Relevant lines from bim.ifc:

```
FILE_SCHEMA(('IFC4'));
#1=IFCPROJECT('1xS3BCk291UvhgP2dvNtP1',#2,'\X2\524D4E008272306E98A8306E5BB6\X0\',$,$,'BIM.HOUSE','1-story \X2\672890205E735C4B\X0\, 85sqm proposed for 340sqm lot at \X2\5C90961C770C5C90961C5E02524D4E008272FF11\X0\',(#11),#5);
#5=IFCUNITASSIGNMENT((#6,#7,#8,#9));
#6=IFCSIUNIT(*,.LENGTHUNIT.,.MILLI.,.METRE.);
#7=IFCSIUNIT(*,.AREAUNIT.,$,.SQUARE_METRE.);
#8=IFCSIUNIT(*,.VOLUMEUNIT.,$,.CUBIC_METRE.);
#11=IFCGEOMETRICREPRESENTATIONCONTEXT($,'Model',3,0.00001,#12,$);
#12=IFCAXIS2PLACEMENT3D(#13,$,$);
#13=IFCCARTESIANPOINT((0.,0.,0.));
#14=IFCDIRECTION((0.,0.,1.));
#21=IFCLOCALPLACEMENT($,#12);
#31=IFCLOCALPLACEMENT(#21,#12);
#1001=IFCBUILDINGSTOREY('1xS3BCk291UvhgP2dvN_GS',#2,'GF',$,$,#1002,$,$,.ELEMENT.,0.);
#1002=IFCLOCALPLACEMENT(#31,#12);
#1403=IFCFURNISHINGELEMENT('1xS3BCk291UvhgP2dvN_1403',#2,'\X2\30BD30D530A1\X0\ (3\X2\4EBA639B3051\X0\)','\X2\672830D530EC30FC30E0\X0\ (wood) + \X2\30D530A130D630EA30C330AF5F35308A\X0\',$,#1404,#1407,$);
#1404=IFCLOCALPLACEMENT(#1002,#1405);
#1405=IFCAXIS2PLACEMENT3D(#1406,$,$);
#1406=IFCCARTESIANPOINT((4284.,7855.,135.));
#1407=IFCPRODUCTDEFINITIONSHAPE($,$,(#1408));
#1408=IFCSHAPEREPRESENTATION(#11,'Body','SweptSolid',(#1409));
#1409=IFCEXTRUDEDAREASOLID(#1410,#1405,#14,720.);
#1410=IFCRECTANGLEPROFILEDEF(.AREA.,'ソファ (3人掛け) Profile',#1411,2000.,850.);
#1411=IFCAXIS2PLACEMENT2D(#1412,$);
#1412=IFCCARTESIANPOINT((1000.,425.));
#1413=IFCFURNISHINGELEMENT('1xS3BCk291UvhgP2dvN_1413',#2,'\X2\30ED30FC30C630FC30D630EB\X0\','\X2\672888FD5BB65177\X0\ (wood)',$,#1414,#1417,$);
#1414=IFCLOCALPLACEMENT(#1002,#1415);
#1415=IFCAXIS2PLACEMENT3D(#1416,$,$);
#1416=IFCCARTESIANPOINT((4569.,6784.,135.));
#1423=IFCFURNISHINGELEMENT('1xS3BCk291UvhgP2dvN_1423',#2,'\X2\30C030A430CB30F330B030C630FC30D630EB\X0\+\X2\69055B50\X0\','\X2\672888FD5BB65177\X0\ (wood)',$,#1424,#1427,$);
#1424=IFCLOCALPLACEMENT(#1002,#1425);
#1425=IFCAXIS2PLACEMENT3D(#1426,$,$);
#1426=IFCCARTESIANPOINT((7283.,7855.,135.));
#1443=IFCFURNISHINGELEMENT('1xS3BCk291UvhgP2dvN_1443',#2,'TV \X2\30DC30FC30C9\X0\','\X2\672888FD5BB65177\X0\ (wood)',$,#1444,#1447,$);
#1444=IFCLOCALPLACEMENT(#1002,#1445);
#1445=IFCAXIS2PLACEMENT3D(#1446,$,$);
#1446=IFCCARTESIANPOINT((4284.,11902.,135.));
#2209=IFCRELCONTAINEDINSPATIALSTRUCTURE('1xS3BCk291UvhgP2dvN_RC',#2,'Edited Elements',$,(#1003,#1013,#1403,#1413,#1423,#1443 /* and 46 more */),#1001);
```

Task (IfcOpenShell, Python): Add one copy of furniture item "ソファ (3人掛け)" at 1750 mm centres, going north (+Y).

```python
import numpy as np
import ifcopenshell
import ifcopenshell.api.geometry
import ifcopenshell.api.root
import ifcopenshell.util.element
import ifcopenshell.util.placement
import ifcopenshell.util.unit

model = ifcopenshell.open("bim.ifc")
unit_scale = ifcopenshell.util.unit.calculate_unit_scale(model)


def reuse_history(source, copy):
    """copy_class also copies each property set's owner history, people and application; keep the originals."""
    for rel in copy.IsDefinedBy:
        if rel.is_a("IfcRelDefinesByProperties") and (history := rel.RelatingPropertyDefinition.OwnerHistory):
            rel.RelatingPropertyDefinition.OwnerHistory = source.OwnerHistory
            ifcopenshell.util.element.remove_deep2(model, history)


source = model.by_id(1403)
base = ifcopenshell.util.placement.get_local_placement(source.ObjectPlacement)
step = np.array([0.0, 1.0, 0.0]) * 1.75 / unit_scale

for i in range(1, 2):
    copy = ifcopenshell.api.root.copy_class(model, product=source)
    copy.Representation = ifcopenshell.util.element.copy_deep(
        model, source.Representation, exclude=["IfcGeometricRepresentationContext", "IfcRepresentationMap"]
    )
    reuse_history(source, copy)
    matrix = base.copy()
    matrix[:3, 3] += i * step
    print("added at", matrix[:3, 3].round(3) + 0.0)
    ifcopenshell.api.geometry.edit_object_placement(model, product=copy, matrix=matrix, is_si=False)

model.write("bim_v2.ifc")
```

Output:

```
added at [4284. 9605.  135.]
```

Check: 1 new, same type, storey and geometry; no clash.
